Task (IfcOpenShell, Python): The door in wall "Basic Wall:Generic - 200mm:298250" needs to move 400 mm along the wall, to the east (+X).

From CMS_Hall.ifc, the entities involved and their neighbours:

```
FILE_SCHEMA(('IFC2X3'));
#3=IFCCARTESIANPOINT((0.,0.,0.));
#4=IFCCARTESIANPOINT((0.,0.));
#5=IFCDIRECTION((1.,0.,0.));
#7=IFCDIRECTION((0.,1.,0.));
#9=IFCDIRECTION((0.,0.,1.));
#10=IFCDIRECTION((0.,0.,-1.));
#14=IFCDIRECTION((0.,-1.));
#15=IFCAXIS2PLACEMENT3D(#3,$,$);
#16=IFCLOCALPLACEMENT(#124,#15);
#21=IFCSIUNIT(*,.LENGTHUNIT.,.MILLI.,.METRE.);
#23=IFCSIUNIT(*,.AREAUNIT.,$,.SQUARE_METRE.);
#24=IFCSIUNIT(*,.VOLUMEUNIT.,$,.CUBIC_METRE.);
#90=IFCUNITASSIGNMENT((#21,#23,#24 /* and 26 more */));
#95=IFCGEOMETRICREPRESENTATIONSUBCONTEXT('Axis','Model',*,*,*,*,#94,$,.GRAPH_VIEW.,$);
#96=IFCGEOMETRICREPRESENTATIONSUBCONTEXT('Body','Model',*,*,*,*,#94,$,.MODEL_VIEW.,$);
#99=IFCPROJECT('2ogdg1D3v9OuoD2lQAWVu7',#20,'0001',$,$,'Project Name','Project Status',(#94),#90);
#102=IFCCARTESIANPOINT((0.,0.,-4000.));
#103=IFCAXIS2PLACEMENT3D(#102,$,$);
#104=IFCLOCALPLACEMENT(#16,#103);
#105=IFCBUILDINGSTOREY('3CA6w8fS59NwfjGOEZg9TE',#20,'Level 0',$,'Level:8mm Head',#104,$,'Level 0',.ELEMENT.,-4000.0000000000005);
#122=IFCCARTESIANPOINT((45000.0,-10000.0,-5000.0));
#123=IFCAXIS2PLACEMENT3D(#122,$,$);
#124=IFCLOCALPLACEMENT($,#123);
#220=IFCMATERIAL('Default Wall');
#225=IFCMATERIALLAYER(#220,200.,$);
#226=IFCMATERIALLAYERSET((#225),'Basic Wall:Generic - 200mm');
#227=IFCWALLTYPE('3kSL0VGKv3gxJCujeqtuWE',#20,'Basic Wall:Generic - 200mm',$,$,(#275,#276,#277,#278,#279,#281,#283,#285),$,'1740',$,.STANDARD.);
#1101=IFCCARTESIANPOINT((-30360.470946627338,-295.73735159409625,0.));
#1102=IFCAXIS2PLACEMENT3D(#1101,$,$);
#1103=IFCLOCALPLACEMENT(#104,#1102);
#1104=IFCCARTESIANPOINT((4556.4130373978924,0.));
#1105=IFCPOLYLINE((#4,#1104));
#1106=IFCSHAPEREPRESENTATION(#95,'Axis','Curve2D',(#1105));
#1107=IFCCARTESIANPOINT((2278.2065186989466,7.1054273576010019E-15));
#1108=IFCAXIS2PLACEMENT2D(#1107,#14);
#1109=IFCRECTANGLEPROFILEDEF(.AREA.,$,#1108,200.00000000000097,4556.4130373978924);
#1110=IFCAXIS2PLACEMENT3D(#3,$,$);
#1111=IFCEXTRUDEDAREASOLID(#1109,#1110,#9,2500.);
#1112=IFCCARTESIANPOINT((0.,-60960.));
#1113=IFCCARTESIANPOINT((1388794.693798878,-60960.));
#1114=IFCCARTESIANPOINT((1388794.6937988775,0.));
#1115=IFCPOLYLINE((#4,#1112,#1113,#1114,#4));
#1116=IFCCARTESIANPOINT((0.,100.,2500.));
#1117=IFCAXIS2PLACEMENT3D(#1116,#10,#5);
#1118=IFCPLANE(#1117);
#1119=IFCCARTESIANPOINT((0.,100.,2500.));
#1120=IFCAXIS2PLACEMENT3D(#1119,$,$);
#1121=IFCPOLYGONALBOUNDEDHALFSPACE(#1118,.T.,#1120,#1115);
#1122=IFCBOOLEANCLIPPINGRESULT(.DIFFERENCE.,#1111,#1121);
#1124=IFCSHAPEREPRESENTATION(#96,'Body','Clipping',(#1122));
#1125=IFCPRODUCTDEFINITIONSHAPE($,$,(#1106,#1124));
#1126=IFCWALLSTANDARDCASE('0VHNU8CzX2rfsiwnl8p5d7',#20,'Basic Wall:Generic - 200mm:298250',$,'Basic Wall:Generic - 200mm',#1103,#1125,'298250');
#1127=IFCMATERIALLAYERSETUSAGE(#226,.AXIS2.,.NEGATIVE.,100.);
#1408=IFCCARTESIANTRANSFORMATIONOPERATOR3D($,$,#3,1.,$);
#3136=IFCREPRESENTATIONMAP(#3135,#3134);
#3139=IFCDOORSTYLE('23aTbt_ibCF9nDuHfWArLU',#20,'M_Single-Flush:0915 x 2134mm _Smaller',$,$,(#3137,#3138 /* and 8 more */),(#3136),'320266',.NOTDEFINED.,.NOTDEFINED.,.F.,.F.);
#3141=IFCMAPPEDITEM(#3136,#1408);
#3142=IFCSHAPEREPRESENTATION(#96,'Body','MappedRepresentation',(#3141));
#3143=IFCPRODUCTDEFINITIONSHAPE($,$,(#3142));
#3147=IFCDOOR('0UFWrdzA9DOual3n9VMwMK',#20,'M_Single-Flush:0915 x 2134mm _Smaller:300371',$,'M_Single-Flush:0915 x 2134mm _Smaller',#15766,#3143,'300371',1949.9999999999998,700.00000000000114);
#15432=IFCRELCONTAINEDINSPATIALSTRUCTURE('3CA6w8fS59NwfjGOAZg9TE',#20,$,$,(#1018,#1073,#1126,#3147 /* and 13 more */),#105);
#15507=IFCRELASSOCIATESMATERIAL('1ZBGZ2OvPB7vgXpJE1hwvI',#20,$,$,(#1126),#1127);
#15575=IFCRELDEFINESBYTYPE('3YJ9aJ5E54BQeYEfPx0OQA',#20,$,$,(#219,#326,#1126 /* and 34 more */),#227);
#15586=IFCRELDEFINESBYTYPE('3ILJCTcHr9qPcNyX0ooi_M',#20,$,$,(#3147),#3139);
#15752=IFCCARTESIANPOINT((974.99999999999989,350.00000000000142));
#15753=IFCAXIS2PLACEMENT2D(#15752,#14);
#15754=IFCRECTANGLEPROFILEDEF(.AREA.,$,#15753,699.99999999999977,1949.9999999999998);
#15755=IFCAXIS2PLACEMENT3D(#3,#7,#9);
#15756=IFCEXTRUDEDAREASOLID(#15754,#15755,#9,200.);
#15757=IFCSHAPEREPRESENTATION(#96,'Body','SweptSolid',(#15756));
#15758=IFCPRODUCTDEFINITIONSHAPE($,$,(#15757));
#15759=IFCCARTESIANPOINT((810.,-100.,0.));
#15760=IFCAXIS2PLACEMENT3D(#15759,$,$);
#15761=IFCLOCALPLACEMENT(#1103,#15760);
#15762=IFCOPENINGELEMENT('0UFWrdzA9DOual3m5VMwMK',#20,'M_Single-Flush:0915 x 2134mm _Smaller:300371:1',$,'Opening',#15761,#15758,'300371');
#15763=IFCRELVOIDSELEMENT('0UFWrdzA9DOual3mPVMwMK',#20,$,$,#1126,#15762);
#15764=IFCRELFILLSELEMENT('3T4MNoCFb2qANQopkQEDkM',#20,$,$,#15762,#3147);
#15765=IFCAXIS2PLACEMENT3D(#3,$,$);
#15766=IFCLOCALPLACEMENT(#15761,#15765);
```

```python
import ifcopenshell
import ifcopenshell.api.geometry
import ifcopenshell.util.placement
import ifcopenshell.util.unit

model = ifcopenshell.open("CMS_Hall.ifc")
unit_scale = ifcopenshell.util.unit.calculate_unit_scale(model)

door = model.by_guid("0UFWrdzA9DOual3n9VMwMK")
opening = door.FillsVoids[0].RelatingOpeningElement
wall = opening.VoidsElements[0].RelatingBuildingElement

wall_matrix = ifcopenshell.util.placement.get_local_placement(wall.ObjectPlacement)
shift = wall_matrix[:3, 0] * 0.4 / unit_scale
before = ifcopenshell.util.placement.get_local_placement(door.ObjectPlacement)[:3, 3].copy()

# The door is placed relative to its opening, so it follows when the opening moves.
matrix = ifcopenshell.util.placement.get_local_placement(opening.ObjectPlacement)
matrix[:3, 3] += shift
ifcopenshell.api.geometry.edit_object_placement(
    model, product=opening, matrix=matrix, is_si=False, should_transform_children=True
)

after = ifcopenshell.util.placement.get_local_placement(door.ObjectPlacement)[:3, 3]
print("door moved by", (after - before).round(3) + 0.0)

model.write("CMS_Hall_edited.ifc")
```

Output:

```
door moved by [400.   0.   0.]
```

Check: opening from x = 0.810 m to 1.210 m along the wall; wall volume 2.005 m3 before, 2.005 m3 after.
